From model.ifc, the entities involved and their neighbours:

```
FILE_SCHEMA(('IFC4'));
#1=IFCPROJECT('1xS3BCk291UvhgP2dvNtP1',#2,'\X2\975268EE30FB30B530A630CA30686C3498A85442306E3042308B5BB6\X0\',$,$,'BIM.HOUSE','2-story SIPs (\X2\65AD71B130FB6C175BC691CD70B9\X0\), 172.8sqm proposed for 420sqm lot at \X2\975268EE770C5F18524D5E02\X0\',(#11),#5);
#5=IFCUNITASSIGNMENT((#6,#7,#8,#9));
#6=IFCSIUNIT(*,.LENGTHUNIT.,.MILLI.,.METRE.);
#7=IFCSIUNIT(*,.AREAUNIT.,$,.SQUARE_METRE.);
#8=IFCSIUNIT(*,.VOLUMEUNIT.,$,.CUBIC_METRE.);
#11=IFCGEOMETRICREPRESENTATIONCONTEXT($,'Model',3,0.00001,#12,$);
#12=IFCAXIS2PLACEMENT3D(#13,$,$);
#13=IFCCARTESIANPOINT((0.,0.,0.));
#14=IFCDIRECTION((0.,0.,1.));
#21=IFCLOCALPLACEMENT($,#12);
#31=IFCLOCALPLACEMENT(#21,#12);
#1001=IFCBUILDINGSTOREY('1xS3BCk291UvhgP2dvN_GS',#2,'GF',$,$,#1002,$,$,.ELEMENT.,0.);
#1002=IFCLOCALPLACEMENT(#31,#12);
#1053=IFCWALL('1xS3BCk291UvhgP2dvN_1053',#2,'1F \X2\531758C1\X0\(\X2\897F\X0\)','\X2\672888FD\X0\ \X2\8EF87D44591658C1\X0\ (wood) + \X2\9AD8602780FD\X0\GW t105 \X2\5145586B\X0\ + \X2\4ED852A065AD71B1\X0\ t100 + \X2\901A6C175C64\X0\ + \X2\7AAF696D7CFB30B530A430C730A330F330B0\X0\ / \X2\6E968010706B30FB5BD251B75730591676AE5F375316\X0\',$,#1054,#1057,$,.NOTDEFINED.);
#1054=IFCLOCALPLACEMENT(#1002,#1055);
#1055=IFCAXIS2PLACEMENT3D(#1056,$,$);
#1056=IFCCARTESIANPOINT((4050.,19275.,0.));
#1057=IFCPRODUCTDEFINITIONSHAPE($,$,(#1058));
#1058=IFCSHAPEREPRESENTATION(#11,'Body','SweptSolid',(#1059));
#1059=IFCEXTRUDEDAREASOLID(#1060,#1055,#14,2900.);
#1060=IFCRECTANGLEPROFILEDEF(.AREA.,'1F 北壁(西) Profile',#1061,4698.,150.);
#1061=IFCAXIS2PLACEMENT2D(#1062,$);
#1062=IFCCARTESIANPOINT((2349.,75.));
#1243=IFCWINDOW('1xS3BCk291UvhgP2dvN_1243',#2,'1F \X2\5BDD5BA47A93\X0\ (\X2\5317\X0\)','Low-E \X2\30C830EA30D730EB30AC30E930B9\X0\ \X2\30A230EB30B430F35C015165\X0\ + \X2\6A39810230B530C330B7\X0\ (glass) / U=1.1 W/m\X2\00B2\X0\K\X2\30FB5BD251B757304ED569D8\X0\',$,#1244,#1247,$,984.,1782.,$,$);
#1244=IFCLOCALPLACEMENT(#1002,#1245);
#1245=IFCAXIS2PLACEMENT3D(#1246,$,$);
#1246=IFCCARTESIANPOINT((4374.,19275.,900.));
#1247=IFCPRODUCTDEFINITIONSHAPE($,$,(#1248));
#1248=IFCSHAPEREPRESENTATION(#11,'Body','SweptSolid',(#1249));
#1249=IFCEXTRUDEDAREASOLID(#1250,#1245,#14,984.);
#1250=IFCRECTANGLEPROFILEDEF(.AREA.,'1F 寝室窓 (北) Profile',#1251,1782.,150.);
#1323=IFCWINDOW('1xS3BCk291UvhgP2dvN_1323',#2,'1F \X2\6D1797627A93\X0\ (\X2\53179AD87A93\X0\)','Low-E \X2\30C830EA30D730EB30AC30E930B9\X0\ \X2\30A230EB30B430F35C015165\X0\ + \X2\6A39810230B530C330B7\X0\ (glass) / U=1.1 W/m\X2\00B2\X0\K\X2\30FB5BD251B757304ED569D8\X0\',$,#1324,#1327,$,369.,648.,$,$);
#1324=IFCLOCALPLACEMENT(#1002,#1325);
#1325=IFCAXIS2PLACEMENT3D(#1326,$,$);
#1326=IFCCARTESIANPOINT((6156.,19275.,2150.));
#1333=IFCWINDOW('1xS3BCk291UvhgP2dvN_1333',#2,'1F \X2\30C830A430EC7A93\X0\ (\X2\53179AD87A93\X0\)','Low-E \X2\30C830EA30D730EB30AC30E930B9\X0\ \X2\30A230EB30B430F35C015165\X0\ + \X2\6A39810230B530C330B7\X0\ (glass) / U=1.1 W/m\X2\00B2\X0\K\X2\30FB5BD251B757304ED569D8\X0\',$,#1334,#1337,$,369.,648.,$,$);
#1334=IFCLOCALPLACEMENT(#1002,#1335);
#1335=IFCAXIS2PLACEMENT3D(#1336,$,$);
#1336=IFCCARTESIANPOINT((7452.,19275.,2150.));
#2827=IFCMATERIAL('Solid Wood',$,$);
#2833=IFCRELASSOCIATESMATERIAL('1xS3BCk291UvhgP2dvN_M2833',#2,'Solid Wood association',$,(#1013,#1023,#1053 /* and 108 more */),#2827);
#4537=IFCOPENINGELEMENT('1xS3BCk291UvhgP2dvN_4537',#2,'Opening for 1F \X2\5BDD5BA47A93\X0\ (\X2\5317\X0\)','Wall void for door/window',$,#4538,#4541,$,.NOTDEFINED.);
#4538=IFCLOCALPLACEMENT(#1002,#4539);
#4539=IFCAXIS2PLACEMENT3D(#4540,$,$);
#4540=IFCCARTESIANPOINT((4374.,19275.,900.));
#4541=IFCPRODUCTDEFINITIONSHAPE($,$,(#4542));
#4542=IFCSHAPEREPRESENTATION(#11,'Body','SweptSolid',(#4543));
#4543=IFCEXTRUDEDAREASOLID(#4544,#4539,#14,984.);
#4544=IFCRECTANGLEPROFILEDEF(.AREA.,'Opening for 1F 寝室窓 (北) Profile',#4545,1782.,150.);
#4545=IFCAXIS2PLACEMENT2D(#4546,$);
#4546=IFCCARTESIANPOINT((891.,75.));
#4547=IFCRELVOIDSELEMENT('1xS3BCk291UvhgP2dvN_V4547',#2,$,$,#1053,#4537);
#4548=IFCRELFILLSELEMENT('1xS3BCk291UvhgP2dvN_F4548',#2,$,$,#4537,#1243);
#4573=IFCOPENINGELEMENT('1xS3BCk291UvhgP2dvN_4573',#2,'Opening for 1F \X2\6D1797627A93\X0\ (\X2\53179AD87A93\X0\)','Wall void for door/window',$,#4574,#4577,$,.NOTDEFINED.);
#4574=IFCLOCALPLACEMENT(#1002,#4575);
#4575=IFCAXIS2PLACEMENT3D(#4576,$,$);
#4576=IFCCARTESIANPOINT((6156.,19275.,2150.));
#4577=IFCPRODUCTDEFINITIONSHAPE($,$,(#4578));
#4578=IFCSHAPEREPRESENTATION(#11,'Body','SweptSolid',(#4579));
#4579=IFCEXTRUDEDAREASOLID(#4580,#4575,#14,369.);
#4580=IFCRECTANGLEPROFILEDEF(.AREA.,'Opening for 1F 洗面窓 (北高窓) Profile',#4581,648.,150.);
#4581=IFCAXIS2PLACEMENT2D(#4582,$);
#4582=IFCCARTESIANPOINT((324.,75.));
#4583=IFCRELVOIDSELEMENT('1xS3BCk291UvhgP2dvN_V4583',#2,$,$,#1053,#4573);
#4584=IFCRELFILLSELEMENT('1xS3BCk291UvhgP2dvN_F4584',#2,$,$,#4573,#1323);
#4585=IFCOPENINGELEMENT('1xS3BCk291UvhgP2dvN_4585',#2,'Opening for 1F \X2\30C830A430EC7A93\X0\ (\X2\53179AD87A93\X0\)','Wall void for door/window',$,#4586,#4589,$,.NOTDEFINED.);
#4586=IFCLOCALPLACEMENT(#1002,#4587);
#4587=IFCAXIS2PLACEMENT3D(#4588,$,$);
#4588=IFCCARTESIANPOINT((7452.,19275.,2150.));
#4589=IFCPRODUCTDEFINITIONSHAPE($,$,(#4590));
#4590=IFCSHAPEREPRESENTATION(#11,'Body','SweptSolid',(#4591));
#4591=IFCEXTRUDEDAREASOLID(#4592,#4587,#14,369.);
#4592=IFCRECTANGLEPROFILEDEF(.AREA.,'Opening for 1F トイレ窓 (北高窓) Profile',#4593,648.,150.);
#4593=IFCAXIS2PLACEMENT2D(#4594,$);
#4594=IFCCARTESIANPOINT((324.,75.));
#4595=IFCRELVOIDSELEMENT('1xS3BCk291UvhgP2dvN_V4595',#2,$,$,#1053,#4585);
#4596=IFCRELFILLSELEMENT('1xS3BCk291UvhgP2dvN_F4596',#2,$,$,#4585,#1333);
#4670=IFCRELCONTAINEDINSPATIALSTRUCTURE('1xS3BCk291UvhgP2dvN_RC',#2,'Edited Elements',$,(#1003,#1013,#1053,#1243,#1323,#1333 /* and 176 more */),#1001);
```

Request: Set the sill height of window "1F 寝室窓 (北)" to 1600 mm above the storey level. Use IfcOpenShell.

```python
import numpy as np
import ifcopenshell
import ifcopenshell.api.geometry
import ifcopenshell.geom
import ifcopenshell.util.element
import ifcopenshell.util.placement
import ifcopenshell.util.shape
import ifcopenshell.util.unit

model = ifcopenshell.open("model.ifc")
unit_scale = ifcopenshell.util.unit.calculate_unit_scale(model)

window = model.by_id(1243)
opening = window.FillsVoids[0].RelatingOpeningElement
storey = ifcopenshell.util.element.get_container(window, ifc_class="IfcBuildingStorey")
level = ifcopenshell.util.placement.get_local_placement(storey.ObjectPlacement)[2, 3]

# The opening's origin need not be at the sill, so measure its lowest point.
shape = ifcopenshell.geom.create_shape(ifcopenshell.geom.settings(), opening)
bottom = ifcopenshell.util.shape.get_shape_bottom_elevation(shape, shape.geometry) / unit_scale
dz = level + 1.6 / unit_scale - bottom

shift = np.array([0.0, 0.0, dz])
# The window is not placed relative to its opening, so move both.
for product in (opening, window):
    matrix = ifcopenshell.util.placement.get_local_placement(product.ObjectPlacement)
    matrix[:3, 3] += shift
    ifcopenshell.api.geometry.edit_object_placement(model, product=product, matrix=matrix, is_si=False)

print(f"moved by {dz * unit_scale:+.3f} m")

model.write("model_v2.ifc")
```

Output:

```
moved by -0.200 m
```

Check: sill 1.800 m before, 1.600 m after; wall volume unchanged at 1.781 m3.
